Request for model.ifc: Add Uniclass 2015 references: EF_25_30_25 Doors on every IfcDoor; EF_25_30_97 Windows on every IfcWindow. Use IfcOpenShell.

First a look at what the model holds.

```python
import ifcopenshell

model = ifcopenshell.open("model.ifc")
print(model.schema)
print("classifications:", [c.Name for c in model.by_type("IfcClassification")])
for ifc_class in ("IfcDoor", "IfcRoof", "IfcStair", "IfcWall", "IfcWindow"):
    print(ifc_class, len(model.by_type(ifc_class)))
```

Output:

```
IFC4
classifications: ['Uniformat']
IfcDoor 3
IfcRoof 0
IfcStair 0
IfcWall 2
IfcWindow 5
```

```python
import ifcopenshell
import ifcopenshell.api.classification

model = ifcopenshell.open("model.ifc")

system = ifcopenshell.api.classification.add_classification(model, classification="Uniclass 2015")

codes = {
    "IfcDoor": ("EF_25_30_25", "Doors"),
    "IfcWindow": ("EF_25_30_97", "Windows"),
}
for ifc_class, (code, name) in codes.items():
    products = model.by_type(ifc_class)
    ifcopenshell.api.classification.add_reference(
        model, products=products, classification=system, identification=code, name=name
    )
    print(code, len(products))

model.write("model_v2.ifc")
```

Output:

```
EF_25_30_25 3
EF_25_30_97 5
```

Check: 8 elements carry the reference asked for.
